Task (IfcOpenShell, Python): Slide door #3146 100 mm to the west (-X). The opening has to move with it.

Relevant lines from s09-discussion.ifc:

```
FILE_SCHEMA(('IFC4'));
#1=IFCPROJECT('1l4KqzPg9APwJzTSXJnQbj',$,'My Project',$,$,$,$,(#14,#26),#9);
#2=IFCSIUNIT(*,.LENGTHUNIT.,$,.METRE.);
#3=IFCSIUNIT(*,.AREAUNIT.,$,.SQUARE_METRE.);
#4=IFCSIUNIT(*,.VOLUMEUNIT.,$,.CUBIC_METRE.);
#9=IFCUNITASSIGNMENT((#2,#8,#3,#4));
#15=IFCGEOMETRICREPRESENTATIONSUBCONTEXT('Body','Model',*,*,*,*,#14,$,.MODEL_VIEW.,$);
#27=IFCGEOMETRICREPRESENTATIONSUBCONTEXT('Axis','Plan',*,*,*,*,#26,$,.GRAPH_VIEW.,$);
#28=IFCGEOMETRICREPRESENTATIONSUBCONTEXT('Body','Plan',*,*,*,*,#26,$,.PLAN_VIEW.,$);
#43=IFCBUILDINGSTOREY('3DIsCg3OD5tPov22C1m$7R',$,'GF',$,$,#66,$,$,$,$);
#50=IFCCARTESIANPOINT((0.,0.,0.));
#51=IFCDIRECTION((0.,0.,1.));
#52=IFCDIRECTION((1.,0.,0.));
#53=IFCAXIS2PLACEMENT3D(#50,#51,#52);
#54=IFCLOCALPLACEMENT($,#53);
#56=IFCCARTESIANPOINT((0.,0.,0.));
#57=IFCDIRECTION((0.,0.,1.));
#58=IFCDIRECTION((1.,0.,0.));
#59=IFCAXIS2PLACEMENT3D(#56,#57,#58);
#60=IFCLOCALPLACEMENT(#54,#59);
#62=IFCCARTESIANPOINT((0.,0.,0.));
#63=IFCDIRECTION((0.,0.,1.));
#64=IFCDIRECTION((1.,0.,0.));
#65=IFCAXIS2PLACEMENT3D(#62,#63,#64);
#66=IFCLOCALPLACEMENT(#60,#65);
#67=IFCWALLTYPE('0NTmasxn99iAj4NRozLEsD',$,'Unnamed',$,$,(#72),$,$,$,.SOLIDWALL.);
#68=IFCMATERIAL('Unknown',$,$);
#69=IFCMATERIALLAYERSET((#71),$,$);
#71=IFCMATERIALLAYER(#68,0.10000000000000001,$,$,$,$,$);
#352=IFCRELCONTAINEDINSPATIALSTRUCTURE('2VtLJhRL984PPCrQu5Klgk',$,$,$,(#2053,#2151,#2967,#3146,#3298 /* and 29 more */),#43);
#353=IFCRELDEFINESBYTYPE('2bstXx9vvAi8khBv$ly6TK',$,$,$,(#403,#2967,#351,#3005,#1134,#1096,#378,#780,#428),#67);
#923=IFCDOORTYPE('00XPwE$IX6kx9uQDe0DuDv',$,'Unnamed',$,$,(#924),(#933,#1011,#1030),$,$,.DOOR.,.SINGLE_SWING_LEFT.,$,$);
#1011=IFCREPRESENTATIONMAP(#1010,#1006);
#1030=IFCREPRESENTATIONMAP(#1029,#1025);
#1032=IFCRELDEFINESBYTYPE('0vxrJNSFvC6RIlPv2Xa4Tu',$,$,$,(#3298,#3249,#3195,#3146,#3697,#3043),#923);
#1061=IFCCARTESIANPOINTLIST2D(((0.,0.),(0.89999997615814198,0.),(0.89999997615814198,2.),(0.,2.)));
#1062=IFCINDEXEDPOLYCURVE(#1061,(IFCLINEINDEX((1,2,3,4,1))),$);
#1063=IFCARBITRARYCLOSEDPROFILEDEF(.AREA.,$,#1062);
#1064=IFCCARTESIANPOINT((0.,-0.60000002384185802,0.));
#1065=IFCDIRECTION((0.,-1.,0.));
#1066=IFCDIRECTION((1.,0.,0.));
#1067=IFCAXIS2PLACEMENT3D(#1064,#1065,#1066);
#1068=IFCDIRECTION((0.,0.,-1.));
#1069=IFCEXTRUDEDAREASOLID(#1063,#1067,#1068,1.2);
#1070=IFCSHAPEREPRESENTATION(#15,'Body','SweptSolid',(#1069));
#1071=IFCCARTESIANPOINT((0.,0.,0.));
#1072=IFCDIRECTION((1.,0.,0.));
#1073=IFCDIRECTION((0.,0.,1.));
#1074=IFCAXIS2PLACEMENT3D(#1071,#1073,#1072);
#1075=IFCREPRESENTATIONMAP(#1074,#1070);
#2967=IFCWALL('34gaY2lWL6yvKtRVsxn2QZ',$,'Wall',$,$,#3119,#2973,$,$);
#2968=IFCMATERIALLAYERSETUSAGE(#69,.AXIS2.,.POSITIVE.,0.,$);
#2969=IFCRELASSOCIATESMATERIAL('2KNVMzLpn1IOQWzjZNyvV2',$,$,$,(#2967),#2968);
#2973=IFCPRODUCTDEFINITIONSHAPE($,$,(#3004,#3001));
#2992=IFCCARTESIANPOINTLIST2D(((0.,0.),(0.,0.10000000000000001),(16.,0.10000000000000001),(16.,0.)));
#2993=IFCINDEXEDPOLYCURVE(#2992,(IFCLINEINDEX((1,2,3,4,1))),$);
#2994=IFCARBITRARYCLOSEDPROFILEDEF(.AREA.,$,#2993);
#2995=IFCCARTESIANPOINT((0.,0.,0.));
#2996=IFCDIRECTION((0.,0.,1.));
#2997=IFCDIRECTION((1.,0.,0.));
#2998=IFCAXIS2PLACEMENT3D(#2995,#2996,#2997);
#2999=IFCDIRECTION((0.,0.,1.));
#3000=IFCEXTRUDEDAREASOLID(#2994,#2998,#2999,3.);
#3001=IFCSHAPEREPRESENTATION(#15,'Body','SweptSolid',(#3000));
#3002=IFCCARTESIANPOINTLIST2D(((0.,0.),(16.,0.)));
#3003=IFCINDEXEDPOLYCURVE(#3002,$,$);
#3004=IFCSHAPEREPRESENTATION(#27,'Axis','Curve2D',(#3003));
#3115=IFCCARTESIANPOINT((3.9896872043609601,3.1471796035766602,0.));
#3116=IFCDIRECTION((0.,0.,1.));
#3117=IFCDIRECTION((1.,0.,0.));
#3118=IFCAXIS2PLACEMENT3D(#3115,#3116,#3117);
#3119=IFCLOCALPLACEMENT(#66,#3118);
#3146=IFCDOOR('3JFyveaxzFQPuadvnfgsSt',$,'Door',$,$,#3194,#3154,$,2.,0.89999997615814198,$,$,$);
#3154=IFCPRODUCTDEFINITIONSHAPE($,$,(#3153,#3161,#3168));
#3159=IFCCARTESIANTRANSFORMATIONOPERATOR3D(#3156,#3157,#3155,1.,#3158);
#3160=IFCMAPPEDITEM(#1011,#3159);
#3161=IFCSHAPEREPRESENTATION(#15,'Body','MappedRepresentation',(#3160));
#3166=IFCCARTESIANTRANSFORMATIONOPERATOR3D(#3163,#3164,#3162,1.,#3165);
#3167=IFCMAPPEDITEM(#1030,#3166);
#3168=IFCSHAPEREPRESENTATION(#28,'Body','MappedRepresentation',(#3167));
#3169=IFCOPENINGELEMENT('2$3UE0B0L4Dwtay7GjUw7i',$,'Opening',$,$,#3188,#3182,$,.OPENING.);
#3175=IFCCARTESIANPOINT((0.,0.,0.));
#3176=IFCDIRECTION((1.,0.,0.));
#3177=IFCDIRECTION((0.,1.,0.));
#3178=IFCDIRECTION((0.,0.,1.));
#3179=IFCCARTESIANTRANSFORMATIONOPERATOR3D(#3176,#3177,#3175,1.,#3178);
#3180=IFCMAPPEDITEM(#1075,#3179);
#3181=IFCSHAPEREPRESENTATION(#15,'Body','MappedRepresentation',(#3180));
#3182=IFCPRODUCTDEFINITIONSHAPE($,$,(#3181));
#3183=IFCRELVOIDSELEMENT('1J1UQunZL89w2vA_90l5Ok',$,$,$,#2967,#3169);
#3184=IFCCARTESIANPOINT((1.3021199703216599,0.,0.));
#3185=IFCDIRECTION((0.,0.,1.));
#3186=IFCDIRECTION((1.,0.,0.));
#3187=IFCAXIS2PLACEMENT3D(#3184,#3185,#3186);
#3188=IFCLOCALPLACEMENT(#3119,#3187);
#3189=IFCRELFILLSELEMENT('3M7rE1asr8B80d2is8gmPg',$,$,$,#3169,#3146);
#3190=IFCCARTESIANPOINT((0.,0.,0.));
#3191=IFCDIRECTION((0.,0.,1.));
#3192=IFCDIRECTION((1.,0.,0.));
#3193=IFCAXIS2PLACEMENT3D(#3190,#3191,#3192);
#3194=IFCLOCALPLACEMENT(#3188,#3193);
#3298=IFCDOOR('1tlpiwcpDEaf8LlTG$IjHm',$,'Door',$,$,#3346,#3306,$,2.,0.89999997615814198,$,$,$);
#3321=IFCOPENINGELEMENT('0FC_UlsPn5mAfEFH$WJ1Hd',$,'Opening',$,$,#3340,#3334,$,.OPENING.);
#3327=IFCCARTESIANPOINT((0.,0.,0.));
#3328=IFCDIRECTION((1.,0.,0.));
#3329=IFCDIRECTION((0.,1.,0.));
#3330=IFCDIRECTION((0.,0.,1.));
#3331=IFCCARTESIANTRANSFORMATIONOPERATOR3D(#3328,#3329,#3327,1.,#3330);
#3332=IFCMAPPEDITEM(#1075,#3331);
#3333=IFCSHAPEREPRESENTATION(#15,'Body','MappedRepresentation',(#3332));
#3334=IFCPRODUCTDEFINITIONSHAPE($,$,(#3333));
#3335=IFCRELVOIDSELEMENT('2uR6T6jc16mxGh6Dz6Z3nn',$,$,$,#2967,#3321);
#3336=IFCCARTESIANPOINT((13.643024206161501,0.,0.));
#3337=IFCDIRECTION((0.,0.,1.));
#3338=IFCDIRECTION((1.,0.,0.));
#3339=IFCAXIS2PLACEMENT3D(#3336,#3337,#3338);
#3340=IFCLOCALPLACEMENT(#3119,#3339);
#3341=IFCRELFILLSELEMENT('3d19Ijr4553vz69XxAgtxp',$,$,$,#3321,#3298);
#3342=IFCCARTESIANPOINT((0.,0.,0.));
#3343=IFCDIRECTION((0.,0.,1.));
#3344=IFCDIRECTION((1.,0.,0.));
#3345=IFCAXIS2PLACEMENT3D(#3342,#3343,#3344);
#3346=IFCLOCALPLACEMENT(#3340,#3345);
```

```python
import ifcopenshell
import ifcopenshell.api.geometry
import ifcopenshell.util.placement
import ifcopenshell.util.unit

model = ifcopenshell.open("s09-discussion.ifc")
unit_scale = ifcopenshell.util.unit.calculate_unit_scale(model)

door = model.by_guid("3JFyveaxzFQPuadvnfgsSt")
opening = door.FillsVoids[0].RelatingOpeningElement
wall = opening.VoidsElements[0].RelatingBuildingElement

wall_matrix = ifcopenshell.util.placement.get_local_placement(wall.ObjectPlacement)
shift = wall_matrix[:3, 0] * -0.1 / unit_scale
before = ifcopenshell.util.placement.get_local_placement(door.ObjectPlacement)[:3, 3].copy()

# The door is placed relative to its opening, so it follows when the opening moves.
matrix = ifcopenshell.util.placement.get_local_placement(opening.ObjectPlacement)
matrix[:3, 3] += shift
ifcopenshell.api.geometry.edit_object_placement(
    model, product=opening, matrix=matrix, is_si=False, should_transform_children=True
)

after = ifcopenshell.util.placement.get_local_placement(door.ObjectPlacement)[:3, 3]
print("door moved by", (after - before).round(3) + 0.0)

model.write("s09-discussion-out.ifc")
```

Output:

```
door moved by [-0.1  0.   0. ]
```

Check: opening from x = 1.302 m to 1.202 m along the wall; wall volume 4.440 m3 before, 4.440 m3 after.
